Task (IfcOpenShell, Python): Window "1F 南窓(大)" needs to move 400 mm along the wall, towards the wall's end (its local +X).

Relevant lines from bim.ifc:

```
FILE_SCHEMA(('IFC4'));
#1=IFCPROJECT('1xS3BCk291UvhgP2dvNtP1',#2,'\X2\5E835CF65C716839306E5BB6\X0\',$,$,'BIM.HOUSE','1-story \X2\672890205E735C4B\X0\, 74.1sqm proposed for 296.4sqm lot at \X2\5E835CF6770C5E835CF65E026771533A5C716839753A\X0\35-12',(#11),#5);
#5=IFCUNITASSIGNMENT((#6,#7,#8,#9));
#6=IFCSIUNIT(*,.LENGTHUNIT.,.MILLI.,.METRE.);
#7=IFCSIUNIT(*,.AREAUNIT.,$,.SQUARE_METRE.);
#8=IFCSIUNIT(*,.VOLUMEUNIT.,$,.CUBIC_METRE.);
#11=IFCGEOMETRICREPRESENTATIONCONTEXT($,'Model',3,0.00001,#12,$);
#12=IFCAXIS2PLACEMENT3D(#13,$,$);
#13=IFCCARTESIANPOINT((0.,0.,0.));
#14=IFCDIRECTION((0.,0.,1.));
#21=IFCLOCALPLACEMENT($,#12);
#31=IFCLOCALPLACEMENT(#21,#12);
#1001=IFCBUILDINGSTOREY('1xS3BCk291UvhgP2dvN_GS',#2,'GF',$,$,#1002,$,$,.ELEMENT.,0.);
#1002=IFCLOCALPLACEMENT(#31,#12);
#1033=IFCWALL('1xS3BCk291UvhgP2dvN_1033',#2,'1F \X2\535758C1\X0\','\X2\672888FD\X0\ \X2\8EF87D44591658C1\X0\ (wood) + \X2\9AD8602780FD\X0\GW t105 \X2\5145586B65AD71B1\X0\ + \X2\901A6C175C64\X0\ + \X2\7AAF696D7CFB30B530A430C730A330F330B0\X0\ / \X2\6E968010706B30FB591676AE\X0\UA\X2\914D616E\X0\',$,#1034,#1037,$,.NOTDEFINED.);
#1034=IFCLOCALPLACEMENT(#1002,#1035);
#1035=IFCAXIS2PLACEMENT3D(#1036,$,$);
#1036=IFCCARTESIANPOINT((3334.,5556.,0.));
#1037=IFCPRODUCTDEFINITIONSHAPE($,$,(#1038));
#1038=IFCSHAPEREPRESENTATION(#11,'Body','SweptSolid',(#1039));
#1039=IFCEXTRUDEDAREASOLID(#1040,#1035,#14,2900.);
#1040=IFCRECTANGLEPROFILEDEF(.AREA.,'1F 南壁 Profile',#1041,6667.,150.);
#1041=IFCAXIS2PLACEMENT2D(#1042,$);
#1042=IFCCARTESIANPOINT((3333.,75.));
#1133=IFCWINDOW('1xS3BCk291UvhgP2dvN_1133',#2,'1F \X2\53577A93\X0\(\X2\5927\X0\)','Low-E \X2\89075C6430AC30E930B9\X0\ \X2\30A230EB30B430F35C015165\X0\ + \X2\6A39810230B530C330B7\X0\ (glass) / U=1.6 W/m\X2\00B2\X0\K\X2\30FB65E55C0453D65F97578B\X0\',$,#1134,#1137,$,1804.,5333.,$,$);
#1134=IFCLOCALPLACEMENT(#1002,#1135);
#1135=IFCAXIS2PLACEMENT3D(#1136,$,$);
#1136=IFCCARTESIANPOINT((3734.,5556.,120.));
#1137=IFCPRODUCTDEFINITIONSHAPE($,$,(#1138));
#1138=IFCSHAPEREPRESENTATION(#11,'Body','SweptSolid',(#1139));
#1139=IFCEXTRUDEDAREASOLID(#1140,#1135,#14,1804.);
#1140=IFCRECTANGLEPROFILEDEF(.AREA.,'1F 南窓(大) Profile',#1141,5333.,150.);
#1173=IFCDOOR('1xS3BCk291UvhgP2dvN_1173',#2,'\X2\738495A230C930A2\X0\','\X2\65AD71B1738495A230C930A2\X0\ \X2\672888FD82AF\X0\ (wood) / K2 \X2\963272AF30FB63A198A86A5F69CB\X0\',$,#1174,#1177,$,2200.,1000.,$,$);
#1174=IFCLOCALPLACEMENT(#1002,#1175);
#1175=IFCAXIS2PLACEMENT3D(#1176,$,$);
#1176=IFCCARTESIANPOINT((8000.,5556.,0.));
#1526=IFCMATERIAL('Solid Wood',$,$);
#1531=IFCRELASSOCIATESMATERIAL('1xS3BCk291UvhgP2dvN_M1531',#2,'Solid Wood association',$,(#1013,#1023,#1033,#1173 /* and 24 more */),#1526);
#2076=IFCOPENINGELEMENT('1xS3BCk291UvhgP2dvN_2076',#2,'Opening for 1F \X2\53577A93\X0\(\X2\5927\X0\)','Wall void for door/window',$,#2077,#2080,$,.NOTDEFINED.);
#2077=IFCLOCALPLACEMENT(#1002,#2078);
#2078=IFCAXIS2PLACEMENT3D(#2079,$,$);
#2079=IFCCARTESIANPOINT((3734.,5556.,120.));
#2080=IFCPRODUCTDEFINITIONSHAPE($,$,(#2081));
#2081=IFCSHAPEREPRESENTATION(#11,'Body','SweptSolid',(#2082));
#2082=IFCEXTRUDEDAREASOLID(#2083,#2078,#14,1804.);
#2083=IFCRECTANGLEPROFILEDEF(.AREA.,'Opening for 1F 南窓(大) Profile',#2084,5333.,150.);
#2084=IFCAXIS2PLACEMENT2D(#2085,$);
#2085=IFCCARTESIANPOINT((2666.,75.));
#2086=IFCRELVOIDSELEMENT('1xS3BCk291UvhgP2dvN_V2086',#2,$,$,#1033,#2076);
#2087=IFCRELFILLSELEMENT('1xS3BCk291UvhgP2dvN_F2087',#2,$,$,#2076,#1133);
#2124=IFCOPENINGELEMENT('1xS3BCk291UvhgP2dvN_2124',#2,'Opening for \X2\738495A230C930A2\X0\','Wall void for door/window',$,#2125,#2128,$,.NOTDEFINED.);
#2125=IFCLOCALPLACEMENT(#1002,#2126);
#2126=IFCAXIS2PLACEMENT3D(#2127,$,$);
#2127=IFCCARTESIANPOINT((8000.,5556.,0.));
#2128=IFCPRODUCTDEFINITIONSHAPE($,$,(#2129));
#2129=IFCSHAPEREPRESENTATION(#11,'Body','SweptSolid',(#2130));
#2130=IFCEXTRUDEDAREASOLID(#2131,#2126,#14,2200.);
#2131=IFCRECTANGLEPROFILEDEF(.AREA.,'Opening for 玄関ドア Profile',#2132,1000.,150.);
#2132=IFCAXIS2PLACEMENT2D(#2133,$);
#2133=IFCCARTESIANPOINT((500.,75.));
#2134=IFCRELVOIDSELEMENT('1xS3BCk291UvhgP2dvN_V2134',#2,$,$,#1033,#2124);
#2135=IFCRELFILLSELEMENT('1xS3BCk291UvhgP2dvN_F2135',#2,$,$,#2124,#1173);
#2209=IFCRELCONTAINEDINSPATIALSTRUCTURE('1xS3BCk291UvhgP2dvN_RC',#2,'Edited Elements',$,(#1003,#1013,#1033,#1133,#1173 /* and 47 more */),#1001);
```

```python
import ifcopenshell
import ifcopenshell.api.geometry
import ifcopenshell.util.placement
import ifcopenshell.util.unit

model = ifcopenshell.open("bim.ifc")
unit_scale = ifcopenshell.util.unit.calculate_unit_scale(model)

window = model.by_guid("1xS3BCk291UvhgP2dvN_1133")
opening = window.FillsVoids[0].RelatingOpeningElement
wall = opening.VoidsElements[0].RelatingBuildingElement

wall_matrix = ifcopenshell.util.placement.get_local_placement(wall.ObjectPlacement)
shift = wall_matrix[:3, 0] * 0.4 / unit_scale
before = ifcopenshell.util.placement.get_local_placement(window.ObjectPlacement)[:3, 3].copy()

# The window is not placed relative to its opening, so move both.
for product in (opening, window):
    matrix = ifcopenshell.util.placement.get_local_placement(product.ObjectPlacement)
    matrix[:3, 3] += shift
    ifcopenshell.api.geometry.edit_object_placement(model, product=product, matrix=matrix, is_si=False)

after = ifcopenshell.util.placement.get_local_placement(window.ObjectPlacement)[:3, 3]
print("window moved by", (after - before).round(3) + 0.0)

model.write("bim_edited.ifc")
```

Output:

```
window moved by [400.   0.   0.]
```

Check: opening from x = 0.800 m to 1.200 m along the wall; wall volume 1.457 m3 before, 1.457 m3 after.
